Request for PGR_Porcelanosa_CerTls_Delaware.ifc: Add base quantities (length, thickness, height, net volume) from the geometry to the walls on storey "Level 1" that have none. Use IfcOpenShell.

First a look at what the model holds.

```python
import ifcopenshell
import ifcopenshell.util.element
import ifcopenshell.util.unit

model = ifcopenshell.open("PGR_Porcelanosa_CerTls_Delaware.ifc")
print(model.schema)
for unit_type in ("LENGTHUNIT", "AREAUNIT", "VOLUMEUNIT"):
    print(unit_type, ifcopenshell.util.unit.calculate_unit_scale(model, unit_type))
storey = next(s for s in model.by_type("IfcBuildingStorey") if s.Name == "Level 1")
walls = [e for e in ifcopenshell.util.element.get_decomposition(storey) if e.is_a("IfcWall")]
for e in sorted(walls, key=lambda e: e.id()):
    print(e.id(), e.is_a(), e.Name, list(ifcopenshell.util.element.get_psets(e, qtos_only=True)), sep=" | ")
```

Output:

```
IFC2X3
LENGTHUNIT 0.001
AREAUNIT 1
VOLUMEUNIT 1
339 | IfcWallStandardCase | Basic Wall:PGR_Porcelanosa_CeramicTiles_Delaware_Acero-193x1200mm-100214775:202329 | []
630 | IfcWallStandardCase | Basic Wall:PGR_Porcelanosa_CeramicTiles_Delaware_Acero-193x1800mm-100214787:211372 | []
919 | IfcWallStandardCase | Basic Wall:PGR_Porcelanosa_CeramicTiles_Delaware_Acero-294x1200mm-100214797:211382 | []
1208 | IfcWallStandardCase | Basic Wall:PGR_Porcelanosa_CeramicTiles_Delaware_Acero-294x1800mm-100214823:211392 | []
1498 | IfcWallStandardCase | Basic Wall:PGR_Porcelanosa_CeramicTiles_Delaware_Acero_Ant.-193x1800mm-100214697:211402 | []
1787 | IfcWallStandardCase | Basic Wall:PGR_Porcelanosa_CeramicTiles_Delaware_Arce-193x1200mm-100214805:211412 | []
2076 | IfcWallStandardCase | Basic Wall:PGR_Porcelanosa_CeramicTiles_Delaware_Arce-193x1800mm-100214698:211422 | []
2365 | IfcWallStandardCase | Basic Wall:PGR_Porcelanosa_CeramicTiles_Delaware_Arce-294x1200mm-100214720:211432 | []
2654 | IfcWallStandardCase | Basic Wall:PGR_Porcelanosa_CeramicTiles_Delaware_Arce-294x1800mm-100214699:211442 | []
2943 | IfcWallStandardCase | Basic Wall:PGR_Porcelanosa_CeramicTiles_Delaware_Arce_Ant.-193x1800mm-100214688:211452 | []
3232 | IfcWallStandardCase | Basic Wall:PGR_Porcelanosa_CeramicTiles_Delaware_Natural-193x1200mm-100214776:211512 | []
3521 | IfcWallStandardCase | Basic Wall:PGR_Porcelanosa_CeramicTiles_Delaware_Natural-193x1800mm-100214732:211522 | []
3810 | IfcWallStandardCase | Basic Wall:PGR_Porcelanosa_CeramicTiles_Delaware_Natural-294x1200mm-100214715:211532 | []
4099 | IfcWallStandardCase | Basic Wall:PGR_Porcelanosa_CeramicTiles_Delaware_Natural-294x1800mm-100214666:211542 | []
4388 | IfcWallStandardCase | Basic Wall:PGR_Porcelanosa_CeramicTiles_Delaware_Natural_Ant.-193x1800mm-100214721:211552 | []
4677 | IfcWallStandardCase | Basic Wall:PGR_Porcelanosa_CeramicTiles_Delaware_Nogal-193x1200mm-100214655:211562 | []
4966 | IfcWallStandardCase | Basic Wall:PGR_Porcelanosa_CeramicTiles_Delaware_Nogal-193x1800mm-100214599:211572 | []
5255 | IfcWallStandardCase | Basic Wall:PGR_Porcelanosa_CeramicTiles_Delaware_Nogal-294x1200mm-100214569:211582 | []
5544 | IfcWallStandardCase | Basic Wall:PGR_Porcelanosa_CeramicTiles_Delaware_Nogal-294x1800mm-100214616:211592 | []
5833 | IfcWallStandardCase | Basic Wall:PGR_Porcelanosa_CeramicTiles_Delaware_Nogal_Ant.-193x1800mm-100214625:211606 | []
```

```python
import ifcopenshell
import ifcopenshell.api.pset
import ifcopenshell.geom
import ifcopenshell.util.element
import ifcopenshell.util.shape
import ifcopenshell.util.unit

model = ifcopenshell.open("PGR_Porcelanosa_CerTls_Delaware.ifc")
unit_scale = ifcopenshell.util.unit.calculate_unit_scale(model)
volume_scale = ifcopenshell.util.unit.calculate_unit_scale(model, "VOLUMEUNIT")
settings = ifcopenshell.geom.settings()

storey = next(s for s in model.by_type("IfcBuildingStorey") if s.Name == "Level 1")
walls = [e for e in ifcopenshell.util.element.get_decomposition(storey) if e.is_a("IfcWall")]

for e in sorted(walls, key=lambda e: e.id()):
    if ifcopenshell.util.element.get_psets(e, qtos_only=True, should_inherit=False):
        continue
    # Geometry comes back in metres, in the element's own axes.
    shape = ifcopenshell.geom.create_shape(settings, e)
    values = {
        "Length": ifcopenshell.util.shape.get_x(shape.geometry) / unit_scale,
        "Width": ifcopenshell.util.shape.get_y(shape.geometry) / unit_scale,
        "Height": ifcopenshell.util.shape.get_z(shape.geometry) / unit_scale,
        "NetVolume": ifcopenshell.util.shape.get_volume(shape.geometry) / volume_scale,
    }
    qto = ifcopenshell.api.pset.add_qto(model, product=e, name="BaseQuantities")
    ifcopenshell.api.pset.edit_qto(model, qto=qto, properties=values)
    print(e.id(), {k: round(v, 3) for k, v in values.items()})

model.write("PGR_Porcelanosa_CerTls_Delaware_rev.ifc")
```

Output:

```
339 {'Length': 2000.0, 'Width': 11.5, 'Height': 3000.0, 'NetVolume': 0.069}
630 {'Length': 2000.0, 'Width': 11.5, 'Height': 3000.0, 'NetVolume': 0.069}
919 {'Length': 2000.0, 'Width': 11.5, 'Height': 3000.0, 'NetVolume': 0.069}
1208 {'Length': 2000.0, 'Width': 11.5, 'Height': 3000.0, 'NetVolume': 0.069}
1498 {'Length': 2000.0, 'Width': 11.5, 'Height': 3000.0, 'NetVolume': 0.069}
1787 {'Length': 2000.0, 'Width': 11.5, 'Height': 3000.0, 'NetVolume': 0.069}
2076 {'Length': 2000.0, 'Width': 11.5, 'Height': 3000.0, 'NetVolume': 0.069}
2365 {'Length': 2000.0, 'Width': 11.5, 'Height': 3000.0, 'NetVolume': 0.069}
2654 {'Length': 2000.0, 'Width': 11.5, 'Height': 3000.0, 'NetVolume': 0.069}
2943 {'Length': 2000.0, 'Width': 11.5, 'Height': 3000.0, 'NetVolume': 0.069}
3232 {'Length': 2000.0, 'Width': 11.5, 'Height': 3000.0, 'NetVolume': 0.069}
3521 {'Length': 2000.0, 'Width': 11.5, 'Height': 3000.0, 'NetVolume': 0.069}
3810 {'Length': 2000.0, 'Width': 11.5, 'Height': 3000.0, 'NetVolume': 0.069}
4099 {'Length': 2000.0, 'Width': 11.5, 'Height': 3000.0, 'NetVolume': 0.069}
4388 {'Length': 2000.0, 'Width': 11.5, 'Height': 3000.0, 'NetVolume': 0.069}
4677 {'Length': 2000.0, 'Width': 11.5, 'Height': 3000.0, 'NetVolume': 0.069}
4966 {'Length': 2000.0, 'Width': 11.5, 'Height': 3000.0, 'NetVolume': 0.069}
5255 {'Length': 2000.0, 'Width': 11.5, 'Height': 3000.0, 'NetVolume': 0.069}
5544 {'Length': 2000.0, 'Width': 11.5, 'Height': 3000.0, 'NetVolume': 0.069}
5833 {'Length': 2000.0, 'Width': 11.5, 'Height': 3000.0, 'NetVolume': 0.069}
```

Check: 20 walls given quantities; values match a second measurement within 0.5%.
